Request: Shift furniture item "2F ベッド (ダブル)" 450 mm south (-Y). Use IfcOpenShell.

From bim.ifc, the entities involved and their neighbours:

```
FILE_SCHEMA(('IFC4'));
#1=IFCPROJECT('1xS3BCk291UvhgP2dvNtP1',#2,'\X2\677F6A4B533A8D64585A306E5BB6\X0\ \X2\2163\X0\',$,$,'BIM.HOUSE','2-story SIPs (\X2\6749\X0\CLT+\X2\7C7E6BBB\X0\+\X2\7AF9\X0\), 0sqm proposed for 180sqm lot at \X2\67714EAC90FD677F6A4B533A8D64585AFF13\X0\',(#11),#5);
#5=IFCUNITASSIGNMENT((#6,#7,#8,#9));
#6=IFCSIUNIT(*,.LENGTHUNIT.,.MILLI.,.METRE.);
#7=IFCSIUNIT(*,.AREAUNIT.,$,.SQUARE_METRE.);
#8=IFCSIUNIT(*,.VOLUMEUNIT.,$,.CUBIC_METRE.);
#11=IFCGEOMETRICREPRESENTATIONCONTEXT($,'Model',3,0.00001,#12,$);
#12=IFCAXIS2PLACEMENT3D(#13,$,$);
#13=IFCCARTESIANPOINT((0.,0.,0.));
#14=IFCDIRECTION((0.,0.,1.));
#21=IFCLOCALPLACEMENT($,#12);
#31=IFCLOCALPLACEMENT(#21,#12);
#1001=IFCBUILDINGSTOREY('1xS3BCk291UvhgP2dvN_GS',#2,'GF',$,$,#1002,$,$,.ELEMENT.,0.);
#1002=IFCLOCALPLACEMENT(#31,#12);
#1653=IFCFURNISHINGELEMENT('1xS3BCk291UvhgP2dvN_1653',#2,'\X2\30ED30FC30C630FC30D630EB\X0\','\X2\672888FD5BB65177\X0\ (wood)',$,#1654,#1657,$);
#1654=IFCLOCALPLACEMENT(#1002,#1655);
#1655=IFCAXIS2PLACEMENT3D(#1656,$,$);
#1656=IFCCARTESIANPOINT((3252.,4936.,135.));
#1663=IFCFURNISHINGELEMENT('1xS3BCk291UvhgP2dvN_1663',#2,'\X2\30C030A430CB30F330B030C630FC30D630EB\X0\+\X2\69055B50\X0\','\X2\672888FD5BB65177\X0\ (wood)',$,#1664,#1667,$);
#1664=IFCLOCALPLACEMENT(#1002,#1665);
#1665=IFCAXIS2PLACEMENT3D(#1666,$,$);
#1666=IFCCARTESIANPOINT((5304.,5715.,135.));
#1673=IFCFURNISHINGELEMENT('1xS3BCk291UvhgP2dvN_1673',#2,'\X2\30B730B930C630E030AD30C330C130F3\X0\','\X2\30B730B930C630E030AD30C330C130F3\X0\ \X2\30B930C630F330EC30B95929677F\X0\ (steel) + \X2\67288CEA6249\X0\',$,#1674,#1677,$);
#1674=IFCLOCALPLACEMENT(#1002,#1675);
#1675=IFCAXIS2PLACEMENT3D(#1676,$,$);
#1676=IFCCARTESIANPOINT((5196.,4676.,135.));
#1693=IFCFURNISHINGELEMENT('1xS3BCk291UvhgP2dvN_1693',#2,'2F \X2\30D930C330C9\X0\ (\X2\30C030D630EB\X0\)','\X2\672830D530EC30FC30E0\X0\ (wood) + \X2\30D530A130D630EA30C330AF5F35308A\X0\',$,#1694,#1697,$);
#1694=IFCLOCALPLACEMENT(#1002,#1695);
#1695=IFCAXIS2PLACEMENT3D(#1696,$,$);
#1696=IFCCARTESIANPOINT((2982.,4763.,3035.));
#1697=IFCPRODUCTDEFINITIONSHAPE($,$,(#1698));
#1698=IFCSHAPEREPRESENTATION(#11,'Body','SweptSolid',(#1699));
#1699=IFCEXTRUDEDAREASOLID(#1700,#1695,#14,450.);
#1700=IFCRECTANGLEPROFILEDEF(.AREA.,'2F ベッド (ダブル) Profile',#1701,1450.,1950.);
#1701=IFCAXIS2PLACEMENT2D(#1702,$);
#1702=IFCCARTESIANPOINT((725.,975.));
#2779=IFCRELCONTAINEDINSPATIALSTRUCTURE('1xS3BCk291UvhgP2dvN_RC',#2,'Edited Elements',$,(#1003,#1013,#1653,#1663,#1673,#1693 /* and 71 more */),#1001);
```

```python
import ifcopenshell
import ifcopenshell.api.geometry
import ifcopenshell.util.placement

model = ifcopenshell.open("bim.ifc")

item = model.by_guid("1xS3BCk291UvhgP2dvN_1693")
matrix = ifcopenshell.util.placement.get_local_placement(item.ObjectPlacement)
matrix[1, 3] -= 450.0
ifcopenshell.api.geometry.edit_object_placement(model, product=item, matrix=matrix, is_si=False)

print(ifcopenshell.util.placement.get_local_placement(item.ObjectPlacement).round(3) + 0.0)

model.write("bim_rev.ifc")
```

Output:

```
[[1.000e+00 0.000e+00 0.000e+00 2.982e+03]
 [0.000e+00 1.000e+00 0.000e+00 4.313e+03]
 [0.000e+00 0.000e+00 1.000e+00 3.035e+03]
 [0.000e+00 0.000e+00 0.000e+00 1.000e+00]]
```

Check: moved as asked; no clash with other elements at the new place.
